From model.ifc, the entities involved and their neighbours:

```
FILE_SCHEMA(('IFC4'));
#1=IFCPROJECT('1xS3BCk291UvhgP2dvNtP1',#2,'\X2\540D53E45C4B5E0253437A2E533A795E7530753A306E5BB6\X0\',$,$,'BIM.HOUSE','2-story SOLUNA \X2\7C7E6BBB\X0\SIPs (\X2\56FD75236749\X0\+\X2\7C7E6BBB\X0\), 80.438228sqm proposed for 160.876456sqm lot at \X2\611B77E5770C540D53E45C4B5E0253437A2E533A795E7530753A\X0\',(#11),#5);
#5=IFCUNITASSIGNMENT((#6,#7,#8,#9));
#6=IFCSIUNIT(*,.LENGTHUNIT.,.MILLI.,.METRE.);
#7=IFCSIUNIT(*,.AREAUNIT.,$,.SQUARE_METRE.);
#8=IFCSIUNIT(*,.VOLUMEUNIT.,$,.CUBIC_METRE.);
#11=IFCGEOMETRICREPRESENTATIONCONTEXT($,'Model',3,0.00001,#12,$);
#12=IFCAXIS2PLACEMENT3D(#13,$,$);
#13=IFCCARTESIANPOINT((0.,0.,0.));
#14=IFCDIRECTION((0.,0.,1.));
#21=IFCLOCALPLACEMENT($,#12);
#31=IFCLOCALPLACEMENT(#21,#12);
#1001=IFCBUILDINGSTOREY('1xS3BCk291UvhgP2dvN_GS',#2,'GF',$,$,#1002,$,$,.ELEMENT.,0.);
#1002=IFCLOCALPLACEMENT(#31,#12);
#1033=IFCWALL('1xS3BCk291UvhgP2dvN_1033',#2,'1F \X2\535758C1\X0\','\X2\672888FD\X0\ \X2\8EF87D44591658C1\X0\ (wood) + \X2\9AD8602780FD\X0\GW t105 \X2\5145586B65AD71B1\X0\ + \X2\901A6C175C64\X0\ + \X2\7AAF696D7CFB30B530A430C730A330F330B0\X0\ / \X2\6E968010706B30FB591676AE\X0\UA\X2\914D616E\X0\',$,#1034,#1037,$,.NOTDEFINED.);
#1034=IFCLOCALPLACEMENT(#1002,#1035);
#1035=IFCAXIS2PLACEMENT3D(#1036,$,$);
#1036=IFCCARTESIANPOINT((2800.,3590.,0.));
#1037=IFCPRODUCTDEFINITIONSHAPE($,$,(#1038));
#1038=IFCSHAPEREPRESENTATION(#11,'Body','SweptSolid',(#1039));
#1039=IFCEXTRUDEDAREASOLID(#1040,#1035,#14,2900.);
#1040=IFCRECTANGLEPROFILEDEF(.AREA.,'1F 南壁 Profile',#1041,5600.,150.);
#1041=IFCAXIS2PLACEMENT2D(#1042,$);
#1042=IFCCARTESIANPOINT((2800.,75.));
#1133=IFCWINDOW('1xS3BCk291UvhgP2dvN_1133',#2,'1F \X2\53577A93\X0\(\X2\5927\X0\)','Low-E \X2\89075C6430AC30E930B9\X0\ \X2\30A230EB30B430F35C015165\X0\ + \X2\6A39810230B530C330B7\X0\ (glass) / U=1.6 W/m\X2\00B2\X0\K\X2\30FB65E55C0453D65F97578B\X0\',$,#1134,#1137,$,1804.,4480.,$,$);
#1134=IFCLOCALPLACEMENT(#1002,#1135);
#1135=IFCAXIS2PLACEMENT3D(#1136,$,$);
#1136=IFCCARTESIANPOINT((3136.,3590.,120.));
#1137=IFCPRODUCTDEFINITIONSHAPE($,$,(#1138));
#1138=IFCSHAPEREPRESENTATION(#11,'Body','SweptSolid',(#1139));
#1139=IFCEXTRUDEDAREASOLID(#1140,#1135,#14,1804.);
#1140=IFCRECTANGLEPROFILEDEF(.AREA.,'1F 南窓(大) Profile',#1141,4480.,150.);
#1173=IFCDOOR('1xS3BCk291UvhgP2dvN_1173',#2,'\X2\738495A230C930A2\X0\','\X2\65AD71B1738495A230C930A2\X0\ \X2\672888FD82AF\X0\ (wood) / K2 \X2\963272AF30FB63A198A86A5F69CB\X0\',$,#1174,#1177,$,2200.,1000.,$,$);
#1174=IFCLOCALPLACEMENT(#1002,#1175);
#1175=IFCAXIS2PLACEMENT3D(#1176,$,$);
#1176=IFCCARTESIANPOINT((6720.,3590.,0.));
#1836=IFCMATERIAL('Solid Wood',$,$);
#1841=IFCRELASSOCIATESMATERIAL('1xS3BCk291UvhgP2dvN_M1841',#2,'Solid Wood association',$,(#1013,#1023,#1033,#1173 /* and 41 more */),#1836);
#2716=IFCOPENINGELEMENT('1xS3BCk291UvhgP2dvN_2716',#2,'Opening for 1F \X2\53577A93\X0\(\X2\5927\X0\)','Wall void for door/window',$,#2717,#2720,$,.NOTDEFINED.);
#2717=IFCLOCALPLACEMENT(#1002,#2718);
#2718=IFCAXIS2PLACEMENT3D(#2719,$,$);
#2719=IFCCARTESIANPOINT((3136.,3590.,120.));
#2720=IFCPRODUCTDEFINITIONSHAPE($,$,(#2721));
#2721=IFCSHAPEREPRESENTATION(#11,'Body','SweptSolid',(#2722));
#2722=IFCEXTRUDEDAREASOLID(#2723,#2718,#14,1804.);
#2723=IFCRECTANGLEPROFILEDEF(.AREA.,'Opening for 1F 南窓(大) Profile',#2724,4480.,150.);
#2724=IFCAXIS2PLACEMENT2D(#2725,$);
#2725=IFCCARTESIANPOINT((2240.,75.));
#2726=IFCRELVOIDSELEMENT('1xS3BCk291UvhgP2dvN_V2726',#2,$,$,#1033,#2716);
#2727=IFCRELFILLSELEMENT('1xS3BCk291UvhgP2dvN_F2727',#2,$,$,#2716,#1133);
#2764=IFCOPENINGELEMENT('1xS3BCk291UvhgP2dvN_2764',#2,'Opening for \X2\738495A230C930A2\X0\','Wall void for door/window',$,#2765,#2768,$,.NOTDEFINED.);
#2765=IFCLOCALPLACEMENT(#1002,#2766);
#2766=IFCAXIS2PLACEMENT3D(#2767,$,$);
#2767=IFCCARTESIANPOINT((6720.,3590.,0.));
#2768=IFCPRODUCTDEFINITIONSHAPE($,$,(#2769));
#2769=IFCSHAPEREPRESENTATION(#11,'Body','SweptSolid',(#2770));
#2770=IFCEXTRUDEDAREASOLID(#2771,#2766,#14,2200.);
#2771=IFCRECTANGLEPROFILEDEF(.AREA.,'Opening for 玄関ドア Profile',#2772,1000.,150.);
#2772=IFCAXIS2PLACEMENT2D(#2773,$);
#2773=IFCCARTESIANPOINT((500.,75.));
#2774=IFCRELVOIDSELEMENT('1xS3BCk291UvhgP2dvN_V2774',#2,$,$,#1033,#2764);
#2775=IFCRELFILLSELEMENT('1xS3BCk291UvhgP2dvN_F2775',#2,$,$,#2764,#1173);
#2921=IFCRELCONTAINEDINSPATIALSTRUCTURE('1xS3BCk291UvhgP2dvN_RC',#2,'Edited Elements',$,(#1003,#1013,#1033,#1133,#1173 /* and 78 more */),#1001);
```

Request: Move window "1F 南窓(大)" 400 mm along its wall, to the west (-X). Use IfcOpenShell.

```python
import ifcopenshell
import ifcopenshell.api.geometry
import ifcopenshell.util.placement
import ifcopenshell.util.unit

model = ifcopenshell.open("model.ifc")
unit_scale = ifcopenshell.util.unit.calculate_unit_scale(model)

window = model.by_guid("1xS3BCk291UvhgP2dvN_1133")
opening = window.FillsVoids[0].RelatingOpeningElement
wall = opening.VoidsElements[0].RelatingBuildingElement

wall_matrix = ifcopenshell.util.placement.get_local_placement(wall.ObjectPlacement)
shift = wall_matrix[:3, 0] * -0.4 / unit_scale
before = ifcopenshell.util.placement.get_local_placement(window.ObjectPlacement)[:3, 3].copy()

# The window is not placed relative to its opening, so move both.
for product in (opening, window):
    matrix = ifcopenshell.util.placement.get_local_placement(product.ObjectPlacement)
    matrix[:3, 3] += shift
    ifcopenshell.api.geometry.edit_object_placement(model, product=product, matrix=matrix, is_si=False)

after = ifcopenshell.util.placement.get_local_placement(window.ObjectPlacement)[:3, 3]
print("window moved by", (after - before).round(3) + 0.0)

model.write("model_rev.ifc")
```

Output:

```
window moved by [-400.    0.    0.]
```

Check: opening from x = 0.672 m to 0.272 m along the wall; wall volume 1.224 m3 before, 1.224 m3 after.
